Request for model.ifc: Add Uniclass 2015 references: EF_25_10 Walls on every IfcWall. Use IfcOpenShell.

First a look at what the model holds.

```python
import ifcopenshell

model = ifcopenshell.open("model.ifc")
print(model.schema)
print("classifications:", [c.Name for c in model.by_type("IfcClassification")])
for ifc_class in ("IfcDoor", "IfcRoof", "IfcStair", "IfcWall", "IfcWindow"):
    print(ifc_class, len(model.by_type(ifc_class)))
```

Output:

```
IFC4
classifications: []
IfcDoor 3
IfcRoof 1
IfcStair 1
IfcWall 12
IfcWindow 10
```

```python
import ifcopenshell
import ifcopenshell.api.classification

model = ifcopenshell.open("model.ifc")

system = ifcopenshell.api.classification.add_classification(model, classification="Uniclass 2015")

codes = {
    "IfcWall": ("EF_25_10", "Walls"),
}
for ifc_class, (code, name) in codes.items():
    products = model.by_type(ifc_class)
    ifcopenshell.api.classification.add_reference(
        model, products=products, classification=system, identification=code, name=name
    )
    print(code, len(products))

model.write("model_edited.ifc")
```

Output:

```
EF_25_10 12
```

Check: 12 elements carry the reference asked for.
